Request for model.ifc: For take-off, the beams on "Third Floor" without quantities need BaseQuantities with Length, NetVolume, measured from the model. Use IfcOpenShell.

First a look at what the model holds.

```python
import ifcopenshell
import ifcopenshell.util.element
import ifcopenshell.util.unit

model = ifcopenshell.open("model.ifc")
print(model.schema)
for unit_type in ("LENGTHUNIT", "AREAUNIT", "VOLUMEUNIT"):
    print(unit_type, ifcopenshell.util.unit.calculate_unit_scale(model, unit_type))
storey = next(s for s in model.by_type("IfcBuildingStorey") if s.Name == "Third Floor")
beams = [e for e in ifcopenshell.util.element.get_decomposition(storey) if e.is_a("IfcBeam")]
for e in sorted(beams, key=lambda e: e.id()):
    print(e.id(), e.is_a(), e.Name, list(ifcopenshell.util.element.get_psets(e, qtos_only=True)), sep=" | ")
```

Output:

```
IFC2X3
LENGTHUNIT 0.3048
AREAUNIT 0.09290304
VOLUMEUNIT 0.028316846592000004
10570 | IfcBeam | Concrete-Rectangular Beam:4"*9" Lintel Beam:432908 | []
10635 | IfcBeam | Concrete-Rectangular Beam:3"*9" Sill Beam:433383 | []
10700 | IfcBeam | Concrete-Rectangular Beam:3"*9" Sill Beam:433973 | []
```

```python
import ifcopenshell
import ifcopenshell.api.pset
import ifcopenshell.geom
import ifcopenshell.util.element
import ifcopenshell.util.shape
import ifcopenshell.util.unit

model = ifcopenshell.open("model.ifc")
unit_scale = ifcopenshell.util.unit.calculate_unit_scale(model)
volume_scale = ifcopenshell.util.unit.calculate_unit_scale(model, "VOLUMEUNIT")
settings = ifcopenshell.geom.settings()

storey = next(s for s in model.by_type("IfcBuildingStorey") if s.Name == "Third Floor")
beams = [e for e in ifcopenshell.util.element.get_decomposition(storey) if e.is_a("IfcBeam")]

for e in sorted(beams, key=lambda e: e.id()):
    if ifcopenshell.util.element.get_psets(e, qtos_only=True, should_inherit=False):
        continue
    # Geometry comes back in metres, in the element's own axes.
    shape = ifcopenshell.geom.create_shape(settings, e)
    values = {
        "Length": ifcopenshell.util.shape.get_max_xyz(shape.geometry) / unit_scale,
        "NetVolume": ifcopenshell.util.shape.get_volume(shape.geometry) / volume_scale,
    }
    qto = ifcopenshell.api.pset.add_qto(model, product=e, name="BaseQuantities")
    ifcopenshell.api.pset.edit_qto(model, qto=qto, properties=values)
    print(e.id(), {k: round(v, 3) for k, v in values.items()})

model.write("model_v2.ifc")
```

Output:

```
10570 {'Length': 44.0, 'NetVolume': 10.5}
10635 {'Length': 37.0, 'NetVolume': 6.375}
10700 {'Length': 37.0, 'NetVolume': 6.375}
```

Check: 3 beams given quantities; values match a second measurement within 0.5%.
